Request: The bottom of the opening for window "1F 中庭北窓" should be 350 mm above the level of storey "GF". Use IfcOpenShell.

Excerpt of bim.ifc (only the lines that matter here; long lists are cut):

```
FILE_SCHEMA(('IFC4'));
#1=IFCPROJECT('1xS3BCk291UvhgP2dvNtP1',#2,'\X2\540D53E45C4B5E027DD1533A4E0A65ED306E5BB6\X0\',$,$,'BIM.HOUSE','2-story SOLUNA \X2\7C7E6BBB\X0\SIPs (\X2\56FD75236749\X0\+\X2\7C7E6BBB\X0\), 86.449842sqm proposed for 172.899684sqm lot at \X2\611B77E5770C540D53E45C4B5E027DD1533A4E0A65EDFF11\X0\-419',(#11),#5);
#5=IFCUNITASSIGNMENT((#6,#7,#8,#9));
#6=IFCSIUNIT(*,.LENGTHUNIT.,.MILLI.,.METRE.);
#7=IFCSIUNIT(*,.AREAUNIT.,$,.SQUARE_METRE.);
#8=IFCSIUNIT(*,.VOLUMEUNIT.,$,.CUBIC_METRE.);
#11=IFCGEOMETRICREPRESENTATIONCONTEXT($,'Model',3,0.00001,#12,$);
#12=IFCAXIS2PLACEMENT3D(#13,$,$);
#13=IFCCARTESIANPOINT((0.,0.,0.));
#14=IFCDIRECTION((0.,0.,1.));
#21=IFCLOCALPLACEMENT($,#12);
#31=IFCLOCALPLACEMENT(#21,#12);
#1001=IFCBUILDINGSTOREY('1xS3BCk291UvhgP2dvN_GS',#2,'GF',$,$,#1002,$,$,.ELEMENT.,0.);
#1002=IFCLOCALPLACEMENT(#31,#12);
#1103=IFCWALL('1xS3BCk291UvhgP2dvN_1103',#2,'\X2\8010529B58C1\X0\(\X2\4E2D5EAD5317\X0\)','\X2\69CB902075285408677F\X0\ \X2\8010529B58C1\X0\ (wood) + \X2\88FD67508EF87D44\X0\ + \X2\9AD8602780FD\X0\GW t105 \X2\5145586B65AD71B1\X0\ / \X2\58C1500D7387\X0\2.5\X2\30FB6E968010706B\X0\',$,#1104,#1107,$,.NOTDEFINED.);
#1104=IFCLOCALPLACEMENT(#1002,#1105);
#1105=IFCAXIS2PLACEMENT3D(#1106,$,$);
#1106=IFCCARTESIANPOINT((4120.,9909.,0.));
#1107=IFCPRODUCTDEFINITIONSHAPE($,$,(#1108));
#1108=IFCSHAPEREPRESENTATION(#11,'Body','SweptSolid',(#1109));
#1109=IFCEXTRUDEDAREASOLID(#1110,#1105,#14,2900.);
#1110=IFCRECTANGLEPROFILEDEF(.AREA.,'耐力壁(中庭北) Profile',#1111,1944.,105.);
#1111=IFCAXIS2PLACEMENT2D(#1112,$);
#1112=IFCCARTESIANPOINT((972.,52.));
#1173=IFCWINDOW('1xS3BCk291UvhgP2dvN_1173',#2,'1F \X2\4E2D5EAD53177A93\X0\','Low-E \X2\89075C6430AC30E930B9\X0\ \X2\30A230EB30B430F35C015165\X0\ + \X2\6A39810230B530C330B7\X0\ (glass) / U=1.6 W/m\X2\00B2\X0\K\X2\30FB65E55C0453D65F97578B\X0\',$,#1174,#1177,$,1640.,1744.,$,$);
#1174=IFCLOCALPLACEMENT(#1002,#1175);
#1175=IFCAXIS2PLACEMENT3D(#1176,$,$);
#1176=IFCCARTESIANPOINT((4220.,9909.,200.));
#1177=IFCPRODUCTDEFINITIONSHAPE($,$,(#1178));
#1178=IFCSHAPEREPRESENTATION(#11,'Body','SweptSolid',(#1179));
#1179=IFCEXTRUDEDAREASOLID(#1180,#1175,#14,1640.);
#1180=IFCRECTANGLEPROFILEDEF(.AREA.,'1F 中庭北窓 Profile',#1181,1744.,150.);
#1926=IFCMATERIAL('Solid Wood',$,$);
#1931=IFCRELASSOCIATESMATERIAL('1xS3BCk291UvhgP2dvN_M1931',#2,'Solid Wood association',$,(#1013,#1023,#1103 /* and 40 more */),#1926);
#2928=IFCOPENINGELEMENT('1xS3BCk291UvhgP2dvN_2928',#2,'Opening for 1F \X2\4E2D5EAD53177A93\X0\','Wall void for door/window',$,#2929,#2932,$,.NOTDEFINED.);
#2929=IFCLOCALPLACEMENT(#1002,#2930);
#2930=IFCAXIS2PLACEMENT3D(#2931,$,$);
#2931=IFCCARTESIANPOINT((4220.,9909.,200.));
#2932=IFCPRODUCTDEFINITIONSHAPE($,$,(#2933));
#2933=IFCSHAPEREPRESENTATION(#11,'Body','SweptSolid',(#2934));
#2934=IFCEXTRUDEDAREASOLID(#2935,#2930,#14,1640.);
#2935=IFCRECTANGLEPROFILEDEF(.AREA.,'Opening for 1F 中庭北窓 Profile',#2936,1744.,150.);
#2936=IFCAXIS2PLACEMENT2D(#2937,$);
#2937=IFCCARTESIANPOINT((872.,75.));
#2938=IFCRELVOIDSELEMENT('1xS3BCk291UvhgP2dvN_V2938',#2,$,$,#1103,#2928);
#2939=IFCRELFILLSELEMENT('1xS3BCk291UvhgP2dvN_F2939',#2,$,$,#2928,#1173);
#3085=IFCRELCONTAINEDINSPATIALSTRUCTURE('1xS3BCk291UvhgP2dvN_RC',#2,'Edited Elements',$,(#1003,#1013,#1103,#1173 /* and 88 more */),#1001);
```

```python
import numpy as np
import ifcopenshell
import ifcopenshell.api.geometry
import ifcopenshell.geom
import ifcopenshell.util.element
import ifcopenshell.util.placement
import ifcopenshell.util.shape
import ifcopenshell.util.unit

model = ifcopenshell.open("bim.ifc")
unit_scale = ifcopenshell.util.unit.calculate_unit_scale(model)

window = model.by_id(1173)
opening = window.FillsVoids[0].RelatingOpeningElement
storey = ifcopenshell.util.element.get_container(window, ifc_class="IfcBuildingStorey")
level = ifcopenshell.util.placement.get_local_placement(storey.ObjectPlacement)[2, 3]

# The opening's origin need not be at the sill, so measure its lowest point.
shape = ifcopenshell.geom.create_shape(ifcopenshell.geom.settings(), opening)
bottom = ifcopenshell.util.shape.get_shape_bottom_elevation(shape, shape.geometry) / unit_scale
dz = level + 350.0 - bottom

shift = np.array([0.0, 0.0, dz])
# The window is not placed relative to its opening, so move both.
for product in (opening, window):
    matrix = ifcopenshell.util.placement.get_local_placement(product.ObjectPlacement)
    matrix[:3, 3] += shift
    ifcopenshell.api.geometry.edit_object_placement(model, product=product, matrix=matrix, is_si=False)

print(f"moved by {dz * unit_scale:+.3f} m")

model.write("bim_rev.ifc")
```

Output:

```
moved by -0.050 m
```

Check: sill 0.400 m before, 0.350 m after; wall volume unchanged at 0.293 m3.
